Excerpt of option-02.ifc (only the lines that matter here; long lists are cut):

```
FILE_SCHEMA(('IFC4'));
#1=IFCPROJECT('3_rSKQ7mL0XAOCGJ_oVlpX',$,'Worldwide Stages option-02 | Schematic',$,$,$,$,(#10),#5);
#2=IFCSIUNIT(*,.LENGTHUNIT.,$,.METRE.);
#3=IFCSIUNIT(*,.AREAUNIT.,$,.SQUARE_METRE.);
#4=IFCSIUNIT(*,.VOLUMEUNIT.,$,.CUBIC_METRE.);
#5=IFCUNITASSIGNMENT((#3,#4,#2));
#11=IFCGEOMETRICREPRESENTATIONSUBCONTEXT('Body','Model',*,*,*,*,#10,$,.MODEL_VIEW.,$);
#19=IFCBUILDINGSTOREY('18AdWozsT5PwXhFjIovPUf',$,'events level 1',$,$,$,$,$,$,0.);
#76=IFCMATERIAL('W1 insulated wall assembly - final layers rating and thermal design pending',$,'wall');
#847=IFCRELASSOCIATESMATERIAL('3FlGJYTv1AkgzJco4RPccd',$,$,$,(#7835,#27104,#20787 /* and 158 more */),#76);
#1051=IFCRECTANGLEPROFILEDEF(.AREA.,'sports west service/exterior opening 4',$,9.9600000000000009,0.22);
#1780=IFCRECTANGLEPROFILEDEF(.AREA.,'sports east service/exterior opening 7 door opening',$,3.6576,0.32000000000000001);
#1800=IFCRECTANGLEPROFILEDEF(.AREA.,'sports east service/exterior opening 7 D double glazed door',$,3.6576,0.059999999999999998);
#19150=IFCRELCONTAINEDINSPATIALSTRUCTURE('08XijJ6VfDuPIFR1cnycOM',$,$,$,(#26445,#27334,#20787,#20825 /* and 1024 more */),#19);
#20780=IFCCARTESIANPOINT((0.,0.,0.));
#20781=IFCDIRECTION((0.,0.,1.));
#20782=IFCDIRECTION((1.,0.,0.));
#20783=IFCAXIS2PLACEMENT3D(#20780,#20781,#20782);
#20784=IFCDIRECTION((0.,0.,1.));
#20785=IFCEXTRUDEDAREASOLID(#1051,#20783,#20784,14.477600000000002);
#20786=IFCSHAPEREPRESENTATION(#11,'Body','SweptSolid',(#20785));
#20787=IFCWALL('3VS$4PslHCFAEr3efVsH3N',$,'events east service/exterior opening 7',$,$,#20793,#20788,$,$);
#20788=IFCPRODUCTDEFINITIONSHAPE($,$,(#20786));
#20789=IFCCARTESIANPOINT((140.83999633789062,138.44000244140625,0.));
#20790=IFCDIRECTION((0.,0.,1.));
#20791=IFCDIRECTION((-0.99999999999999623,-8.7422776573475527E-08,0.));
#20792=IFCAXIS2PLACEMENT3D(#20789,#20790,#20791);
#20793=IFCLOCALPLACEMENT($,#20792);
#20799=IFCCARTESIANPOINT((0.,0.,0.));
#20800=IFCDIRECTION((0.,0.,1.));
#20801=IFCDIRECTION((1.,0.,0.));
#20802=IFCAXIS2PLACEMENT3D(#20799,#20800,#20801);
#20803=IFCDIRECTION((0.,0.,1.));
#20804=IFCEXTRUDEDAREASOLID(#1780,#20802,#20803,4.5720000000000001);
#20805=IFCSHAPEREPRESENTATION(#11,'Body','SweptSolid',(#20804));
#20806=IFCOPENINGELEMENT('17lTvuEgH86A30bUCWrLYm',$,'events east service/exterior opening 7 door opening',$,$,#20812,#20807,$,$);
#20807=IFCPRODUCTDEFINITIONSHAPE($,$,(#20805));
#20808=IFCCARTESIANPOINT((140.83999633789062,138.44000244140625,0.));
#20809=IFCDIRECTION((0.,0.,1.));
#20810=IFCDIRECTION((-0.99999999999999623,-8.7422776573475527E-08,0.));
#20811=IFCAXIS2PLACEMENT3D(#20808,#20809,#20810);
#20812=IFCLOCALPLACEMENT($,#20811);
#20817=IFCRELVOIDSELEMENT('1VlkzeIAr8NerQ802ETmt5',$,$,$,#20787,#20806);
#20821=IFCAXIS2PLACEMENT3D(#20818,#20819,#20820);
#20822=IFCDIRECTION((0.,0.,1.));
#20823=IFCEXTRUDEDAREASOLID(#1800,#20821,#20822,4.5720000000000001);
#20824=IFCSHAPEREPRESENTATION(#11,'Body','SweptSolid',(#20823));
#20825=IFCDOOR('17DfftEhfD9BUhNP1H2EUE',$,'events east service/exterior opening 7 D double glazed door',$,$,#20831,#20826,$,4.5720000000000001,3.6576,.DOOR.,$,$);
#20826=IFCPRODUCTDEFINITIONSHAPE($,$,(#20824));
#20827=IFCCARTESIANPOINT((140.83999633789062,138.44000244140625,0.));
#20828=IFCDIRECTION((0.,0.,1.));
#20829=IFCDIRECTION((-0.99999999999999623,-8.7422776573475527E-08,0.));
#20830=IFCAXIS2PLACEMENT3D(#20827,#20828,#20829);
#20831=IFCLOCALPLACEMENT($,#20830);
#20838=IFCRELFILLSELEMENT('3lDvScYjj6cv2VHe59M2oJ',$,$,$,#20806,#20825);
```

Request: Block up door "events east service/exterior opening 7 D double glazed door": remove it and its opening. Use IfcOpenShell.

```python
import ifcopenshell
import ifcopenshell.api.feature
import ifcopenshell.api.root
import ifcopenshell.geom
import ifcopenshell.util.shape

model = ifcopenshell.open("option-02.ifc")
settings = ifcopenshell.geom.settings()


def volume(element):
    """Net volume in cubic metres, openings subtracted."""
    shape = ifcopenshell.geom.create_shape(settings, element)
    return ifcopenshell.util.shape.get_volume(shape.geometry)


door = model.by_guid("17DfftEhfD9BUhNP1H2EUE")
opening = door.FillsVoids[0].RelatingOpeningElement
wall = opening.VoidsElements[0].RelatingBuildingElement
before = volume(wall)

ifcopenshell.api.root.remove_product(model, product=door)
ifcopenshell.api.feature.remove_feature(model, feature=opening)

after = volume(wall)

print(f"wall volume {before:.3f} -> {after:.3f} m3")

model.write("option-02_rev.ifc")
```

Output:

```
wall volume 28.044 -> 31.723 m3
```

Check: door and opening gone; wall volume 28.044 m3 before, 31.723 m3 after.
